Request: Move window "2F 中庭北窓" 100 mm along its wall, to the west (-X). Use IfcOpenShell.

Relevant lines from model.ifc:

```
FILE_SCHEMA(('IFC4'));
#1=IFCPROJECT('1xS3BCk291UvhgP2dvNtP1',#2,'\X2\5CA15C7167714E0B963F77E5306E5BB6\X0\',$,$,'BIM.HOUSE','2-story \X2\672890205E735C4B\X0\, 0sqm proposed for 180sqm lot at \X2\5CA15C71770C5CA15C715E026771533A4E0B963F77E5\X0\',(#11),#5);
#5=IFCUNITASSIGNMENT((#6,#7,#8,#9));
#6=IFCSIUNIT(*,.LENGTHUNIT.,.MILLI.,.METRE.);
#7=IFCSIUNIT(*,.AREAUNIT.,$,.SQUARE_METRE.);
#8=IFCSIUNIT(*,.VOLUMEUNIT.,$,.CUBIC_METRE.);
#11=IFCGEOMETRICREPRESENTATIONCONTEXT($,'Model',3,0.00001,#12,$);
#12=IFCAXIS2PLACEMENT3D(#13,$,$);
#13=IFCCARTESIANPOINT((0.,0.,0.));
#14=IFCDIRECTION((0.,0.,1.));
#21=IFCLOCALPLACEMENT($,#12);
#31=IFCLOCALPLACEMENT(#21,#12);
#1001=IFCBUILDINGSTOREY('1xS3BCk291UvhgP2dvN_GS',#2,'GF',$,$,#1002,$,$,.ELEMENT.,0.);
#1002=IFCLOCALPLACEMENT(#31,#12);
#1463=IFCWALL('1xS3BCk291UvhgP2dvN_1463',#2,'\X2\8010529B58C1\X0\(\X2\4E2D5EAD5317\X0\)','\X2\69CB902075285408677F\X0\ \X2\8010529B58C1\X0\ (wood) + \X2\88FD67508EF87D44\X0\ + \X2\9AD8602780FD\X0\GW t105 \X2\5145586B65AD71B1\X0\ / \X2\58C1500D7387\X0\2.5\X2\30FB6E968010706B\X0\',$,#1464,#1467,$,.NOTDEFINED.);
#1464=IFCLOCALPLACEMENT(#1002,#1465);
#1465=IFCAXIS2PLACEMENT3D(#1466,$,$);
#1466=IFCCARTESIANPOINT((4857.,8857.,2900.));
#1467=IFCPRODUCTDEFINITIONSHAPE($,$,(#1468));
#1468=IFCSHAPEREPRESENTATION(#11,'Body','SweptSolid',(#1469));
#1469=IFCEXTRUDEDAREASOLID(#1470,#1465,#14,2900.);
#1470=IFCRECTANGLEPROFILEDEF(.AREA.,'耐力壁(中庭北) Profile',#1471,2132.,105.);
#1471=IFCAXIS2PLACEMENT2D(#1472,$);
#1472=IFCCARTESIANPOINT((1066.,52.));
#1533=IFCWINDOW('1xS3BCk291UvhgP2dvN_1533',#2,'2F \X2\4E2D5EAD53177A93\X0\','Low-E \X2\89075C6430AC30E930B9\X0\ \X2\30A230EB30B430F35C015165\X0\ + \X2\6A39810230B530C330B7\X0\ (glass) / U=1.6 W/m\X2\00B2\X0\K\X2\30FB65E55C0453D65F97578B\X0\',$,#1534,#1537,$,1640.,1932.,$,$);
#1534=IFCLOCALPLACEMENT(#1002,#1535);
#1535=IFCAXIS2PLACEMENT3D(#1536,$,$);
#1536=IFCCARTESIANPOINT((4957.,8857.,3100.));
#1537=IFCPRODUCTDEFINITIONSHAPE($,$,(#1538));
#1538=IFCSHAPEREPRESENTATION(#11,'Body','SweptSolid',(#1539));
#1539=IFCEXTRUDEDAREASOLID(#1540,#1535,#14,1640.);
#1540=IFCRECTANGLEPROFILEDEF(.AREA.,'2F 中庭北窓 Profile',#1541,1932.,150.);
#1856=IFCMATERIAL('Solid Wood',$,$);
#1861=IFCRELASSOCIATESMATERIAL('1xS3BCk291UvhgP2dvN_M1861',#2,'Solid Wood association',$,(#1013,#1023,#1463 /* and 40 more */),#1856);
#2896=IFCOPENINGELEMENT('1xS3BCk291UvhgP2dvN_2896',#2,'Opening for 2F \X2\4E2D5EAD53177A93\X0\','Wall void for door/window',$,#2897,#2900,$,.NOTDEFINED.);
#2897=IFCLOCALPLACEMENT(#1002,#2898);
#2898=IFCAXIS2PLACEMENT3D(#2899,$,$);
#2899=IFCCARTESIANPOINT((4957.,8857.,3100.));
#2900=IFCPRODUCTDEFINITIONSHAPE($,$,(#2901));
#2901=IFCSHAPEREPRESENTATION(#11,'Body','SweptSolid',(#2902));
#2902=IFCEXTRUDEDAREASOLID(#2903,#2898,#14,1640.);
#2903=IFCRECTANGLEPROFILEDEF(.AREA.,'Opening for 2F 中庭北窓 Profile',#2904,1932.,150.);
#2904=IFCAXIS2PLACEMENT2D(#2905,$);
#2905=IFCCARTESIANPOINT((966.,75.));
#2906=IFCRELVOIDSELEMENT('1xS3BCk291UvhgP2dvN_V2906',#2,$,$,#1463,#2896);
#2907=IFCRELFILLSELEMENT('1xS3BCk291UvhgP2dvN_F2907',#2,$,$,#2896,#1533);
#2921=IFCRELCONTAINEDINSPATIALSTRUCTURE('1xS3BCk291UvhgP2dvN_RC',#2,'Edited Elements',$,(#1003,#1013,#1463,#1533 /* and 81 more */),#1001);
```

```python
import ifcopenshell
import ifcopenshell.api.geometry
import ifcopenshell.util.placement
import ifcopenshell.util.unit

model = ifcopenshell.open("model.ifc")
unit_scale = ifcopenshell.util.unit.calculate_unit_scale(model)

window = model.by_guid("1xS3BCk291UvhgP2dvN_1533")
opening = window.FillsVoids[0].RelatingOpeningElement
wall = opening.VoidsElements[0].RelatingBuildingElement

wall_matrix = ifcopenshell.util.placement.get_local_placement(wall.ObjectPlacement)
shift = wall_matrix[:3, 0] * -0.1 / unit_scale
before = ifcopenshell.util.placement.get_local_placement(window.ObjectPlacement)[:3, 3].copy()

# The window is not placed relative to its opening, so move both.
for product in (opening, window):
    matrix = ifcopenshell.util.placement.get_local_placement(product.ObjectPlacement)
    matrix[:3, 3] += shift
    ifcopenshell.api.geometry.edit_object_placement(model, product=product, matrix=matrix, is_si=False)

after = ifcopenshell.util.placement.get_local_placement(window.ObjectPlacement)[:3, 3]
print("window moved by", (after - before).round(3) + 0.0)

model.write("model_v2.ifc")
```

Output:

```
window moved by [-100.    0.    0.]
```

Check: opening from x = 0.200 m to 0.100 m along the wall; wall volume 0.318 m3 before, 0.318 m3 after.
